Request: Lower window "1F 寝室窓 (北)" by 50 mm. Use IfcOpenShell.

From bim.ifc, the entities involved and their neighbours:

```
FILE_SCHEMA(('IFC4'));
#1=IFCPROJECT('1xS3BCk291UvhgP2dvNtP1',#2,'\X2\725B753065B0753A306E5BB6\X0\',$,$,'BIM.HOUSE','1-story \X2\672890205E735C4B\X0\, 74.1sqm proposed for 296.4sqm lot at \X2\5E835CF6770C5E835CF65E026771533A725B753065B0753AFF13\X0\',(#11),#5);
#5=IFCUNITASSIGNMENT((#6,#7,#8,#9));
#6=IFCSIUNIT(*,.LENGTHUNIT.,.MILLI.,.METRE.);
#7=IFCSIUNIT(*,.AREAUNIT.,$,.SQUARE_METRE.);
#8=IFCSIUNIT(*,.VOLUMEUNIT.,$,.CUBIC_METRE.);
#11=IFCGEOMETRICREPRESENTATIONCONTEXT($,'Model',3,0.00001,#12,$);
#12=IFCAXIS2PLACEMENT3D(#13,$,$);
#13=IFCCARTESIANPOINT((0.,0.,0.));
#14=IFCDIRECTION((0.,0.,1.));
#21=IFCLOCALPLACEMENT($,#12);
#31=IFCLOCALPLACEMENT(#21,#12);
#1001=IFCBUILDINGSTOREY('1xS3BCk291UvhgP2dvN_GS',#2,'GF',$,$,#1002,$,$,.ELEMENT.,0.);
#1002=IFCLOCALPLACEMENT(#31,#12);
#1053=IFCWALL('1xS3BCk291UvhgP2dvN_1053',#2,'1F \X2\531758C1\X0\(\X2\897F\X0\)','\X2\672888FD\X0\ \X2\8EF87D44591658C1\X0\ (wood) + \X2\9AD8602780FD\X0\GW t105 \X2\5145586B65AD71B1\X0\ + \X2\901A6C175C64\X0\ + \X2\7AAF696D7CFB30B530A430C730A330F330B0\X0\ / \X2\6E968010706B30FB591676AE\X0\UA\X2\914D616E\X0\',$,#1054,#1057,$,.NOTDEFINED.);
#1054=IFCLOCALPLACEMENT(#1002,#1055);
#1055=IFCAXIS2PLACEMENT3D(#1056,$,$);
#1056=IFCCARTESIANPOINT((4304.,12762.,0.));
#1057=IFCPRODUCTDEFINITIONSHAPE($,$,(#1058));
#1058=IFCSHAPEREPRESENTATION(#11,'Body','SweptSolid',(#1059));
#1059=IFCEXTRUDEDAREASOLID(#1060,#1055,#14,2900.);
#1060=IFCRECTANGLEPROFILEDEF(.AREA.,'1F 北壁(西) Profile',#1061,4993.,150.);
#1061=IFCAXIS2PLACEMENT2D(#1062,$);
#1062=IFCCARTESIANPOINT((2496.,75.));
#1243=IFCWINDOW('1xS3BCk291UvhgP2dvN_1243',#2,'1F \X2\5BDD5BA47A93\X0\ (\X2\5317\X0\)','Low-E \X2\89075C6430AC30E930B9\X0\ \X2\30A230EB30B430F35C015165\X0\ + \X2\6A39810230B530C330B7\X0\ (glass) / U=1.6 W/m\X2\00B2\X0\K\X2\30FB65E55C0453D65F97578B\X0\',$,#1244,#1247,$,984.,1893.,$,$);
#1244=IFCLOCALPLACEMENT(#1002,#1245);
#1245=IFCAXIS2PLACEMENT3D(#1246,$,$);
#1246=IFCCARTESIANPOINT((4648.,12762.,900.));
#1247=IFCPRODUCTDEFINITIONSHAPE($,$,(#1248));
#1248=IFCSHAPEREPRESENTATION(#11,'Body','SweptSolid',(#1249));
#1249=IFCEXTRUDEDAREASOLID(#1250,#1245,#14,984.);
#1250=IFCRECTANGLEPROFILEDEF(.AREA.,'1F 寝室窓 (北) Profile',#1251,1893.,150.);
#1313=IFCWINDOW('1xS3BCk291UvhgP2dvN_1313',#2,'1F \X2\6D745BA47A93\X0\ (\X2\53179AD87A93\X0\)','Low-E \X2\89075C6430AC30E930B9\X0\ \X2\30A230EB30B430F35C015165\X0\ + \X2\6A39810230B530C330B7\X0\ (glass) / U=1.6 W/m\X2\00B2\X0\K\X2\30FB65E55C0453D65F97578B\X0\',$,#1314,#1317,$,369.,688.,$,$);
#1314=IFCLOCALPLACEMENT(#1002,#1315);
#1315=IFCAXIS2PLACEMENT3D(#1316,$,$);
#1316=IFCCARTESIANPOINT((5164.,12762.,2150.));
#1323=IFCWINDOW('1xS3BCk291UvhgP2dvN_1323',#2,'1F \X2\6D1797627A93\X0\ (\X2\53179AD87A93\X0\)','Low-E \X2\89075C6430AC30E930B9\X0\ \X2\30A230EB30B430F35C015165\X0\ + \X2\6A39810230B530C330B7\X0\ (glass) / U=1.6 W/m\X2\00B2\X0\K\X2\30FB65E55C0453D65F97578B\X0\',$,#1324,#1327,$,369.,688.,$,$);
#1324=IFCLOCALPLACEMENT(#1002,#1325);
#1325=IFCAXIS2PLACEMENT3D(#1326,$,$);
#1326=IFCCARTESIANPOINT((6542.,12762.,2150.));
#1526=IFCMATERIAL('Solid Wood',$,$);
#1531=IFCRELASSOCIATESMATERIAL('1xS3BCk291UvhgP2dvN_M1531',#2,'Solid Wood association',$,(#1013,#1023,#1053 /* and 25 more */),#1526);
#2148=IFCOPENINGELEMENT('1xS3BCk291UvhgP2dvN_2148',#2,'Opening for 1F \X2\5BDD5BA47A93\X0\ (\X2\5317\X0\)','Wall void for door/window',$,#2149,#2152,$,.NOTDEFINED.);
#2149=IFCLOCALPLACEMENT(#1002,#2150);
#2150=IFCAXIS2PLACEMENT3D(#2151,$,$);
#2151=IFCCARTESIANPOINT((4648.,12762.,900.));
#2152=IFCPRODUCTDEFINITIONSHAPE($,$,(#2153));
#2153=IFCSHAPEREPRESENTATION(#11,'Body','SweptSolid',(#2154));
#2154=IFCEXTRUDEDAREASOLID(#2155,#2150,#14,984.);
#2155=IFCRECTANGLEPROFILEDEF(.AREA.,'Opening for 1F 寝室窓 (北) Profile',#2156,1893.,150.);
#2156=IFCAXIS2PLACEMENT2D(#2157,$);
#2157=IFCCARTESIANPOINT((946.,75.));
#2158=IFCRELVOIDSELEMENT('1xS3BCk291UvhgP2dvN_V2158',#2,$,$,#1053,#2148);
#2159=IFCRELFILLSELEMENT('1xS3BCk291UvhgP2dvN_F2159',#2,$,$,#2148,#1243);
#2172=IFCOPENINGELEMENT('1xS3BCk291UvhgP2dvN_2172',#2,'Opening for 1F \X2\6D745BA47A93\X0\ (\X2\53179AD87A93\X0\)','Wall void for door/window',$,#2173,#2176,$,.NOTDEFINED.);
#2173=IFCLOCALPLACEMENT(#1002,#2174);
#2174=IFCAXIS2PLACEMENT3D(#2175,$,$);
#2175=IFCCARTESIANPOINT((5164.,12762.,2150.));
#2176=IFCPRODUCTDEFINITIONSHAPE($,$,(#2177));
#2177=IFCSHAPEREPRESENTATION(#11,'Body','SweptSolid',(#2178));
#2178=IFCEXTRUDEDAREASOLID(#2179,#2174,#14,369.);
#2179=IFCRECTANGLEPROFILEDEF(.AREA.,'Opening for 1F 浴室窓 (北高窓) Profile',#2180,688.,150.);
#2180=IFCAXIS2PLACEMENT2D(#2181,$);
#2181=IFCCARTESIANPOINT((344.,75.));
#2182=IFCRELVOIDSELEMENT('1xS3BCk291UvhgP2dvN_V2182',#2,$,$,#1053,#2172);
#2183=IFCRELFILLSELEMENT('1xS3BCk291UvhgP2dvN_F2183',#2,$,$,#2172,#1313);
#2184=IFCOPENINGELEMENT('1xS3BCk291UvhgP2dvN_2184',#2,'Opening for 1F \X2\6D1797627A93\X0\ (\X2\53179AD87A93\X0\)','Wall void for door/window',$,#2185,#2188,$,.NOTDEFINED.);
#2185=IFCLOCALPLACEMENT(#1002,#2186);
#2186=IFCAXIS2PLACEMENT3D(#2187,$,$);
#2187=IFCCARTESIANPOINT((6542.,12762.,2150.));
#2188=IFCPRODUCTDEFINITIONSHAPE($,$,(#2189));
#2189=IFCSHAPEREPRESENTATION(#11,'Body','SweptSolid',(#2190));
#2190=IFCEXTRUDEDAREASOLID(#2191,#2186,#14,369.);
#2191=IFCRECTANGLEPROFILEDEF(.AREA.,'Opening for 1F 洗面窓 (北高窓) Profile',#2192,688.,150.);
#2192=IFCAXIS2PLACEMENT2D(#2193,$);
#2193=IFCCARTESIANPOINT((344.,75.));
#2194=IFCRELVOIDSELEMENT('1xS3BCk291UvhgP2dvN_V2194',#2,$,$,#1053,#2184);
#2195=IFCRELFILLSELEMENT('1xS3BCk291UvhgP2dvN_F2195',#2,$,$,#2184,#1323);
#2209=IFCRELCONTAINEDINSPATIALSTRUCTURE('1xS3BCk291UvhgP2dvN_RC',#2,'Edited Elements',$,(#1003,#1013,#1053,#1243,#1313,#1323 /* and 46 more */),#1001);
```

```python
import numpy as np
import ifcopenshell
import ifcopenshell.api.geometry
import ifcopenshell.util.placement
import ifcopenshell.util.unit

model = ifcopenshell.open("bim.ifc")
unit_scale = ifcopenshell.util.unit.calculate_unit_scale(model)

window = model.by_id(1243)
opening = window.FillsVoids[0].RelatingOpeningElement
dz = -0.05 / unit_scale

shift = np.array([0.0, 0.0, dz])
# The window is not placed relative to its opening, so move both.
for product in (opening, window):
    matrix = ifcopenshell.util.placement.get_local_placement(product.ObjectPlacement)
    matrix[:3, 3] += shift
    ifcopenshell.api.geometry.edit_object_placement(model, product=product, matrix=matrix, is_si=False)

print(f"moved by {dz * unit_scale:+.3f} m")

model.write("bim_rev.ifc")
```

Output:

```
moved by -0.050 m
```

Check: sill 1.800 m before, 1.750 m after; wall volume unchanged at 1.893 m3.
